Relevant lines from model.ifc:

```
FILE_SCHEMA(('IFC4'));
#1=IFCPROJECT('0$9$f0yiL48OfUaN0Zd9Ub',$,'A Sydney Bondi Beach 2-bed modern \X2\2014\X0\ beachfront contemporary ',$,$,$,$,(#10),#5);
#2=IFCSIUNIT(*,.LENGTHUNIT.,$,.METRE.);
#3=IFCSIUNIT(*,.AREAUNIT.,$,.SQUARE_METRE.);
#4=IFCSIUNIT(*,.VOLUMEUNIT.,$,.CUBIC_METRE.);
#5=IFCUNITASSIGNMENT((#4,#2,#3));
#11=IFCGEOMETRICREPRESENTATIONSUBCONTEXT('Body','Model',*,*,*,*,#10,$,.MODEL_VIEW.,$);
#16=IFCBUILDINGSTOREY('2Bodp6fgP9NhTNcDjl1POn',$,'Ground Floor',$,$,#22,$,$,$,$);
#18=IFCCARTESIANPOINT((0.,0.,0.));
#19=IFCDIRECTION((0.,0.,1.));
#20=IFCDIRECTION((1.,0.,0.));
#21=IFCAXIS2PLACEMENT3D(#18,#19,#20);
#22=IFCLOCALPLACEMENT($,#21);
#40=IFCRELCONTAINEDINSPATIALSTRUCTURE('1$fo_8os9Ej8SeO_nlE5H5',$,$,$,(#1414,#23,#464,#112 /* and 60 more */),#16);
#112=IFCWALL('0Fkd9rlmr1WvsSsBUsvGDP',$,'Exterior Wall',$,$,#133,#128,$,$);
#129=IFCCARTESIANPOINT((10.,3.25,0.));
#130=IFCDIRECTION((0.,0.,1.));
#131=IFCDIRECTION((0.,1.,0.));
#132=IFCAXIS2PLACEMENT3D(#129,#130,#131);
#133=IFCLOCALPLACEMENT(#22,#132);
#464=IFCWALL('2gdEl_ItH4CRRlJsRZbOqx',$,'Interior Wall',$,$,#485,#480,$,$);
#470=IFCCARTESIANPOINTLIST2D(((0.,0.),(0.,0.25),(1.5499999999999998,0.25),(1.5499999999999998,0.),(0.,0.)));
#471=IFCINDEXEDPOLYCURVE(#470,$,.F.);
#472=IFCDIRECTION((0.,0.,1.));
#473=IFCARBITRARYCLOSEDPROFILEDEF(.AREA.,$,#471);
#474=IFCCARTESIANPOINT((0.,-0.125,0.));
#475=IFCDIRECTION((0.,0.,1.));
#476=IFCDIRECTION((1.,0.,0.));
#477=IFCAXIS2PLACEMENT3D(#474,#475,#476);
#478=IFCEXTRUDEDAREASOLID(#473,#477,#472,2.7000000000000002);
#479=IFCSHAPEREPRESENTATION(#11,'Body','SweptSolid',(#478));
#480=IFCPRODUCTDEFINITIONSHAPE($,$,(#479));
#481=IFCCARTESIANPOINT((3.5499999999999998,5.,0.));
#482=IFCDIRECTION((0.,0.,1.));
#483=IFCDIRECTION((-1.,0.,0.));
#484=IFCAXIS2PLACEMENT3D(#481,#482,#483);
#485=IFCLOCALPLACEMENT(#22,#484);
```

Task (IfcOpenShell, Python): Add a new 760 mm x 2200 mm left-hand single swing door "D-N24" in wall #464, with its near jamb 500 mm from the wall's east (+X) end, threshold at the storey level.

```python
import numpy as np
import ifcopenshell
import ifcopenshell.api.feature
import ifcopenshell.api.geometry
import ifcopenshell.api.root
import ifcopenshell.api.spatial
import ifcopenshell.geom
import ifcopenshell.util.element
import ifcopenshell.util.placement
import ifcopenshell.util.representation
import ifcopenshell.util.shape
import ifcopenshell.util.unit

model = ifcopenshell.open("model.ifc")
unit_scale = ifcopenshell.util.unit.calculate_unit_scale(model)
settings = ifcopenshell.geom.settings()


def volume(element):
    """Net volume in cubic metres, openings subtracted."""
    shape = ifcopenshell.geom.create_shape(settings, element)
    return ifcopenshell.util.shape.get_volume(shape.geometry)


wall = model.by_guid("2gdEl_ItH4CRRlJsRZbOqx")
storey = ifcopenshell.util.element.get_container(wall, ifc_class="IfcBuildingStorey")
context = ifcopenshell.util.representation.get_context(model, "Model", "Body", "MODEL_VIEW")
before = volume(wall)

width, height, from_end, sill = 0.76, 2.2, 0.5, 0.0  # metres

# The wall runs along its own X axis, and the end named is its -X end.
wall_shape = ifcopenshell.geom.create_shape(settings, wall)
x, y, z = ifcopenshell.util.shape.get_vertices(wall_shape.geometry).T
start = x.min() + from_end
face, thickness = float(y.min()), float(y.max() - y.min())
wall_matrix = ifcopenshell.util.placement.get_local_placement(wall.ObjectPlacement)
level = ifcopenshell.util.placement.get_local_placement(storey.ObjectPlacement)[2, 3]


def in_wall(x, y):
    """Placement at x, y metres in the wall's axes, at sill height."""
    matrix = wall_matrix.copy()
    matrix[:, 3] = wall_matrix @ np.array([x / unit_scale, y / unit_scale, 0.0, 1.0])
    matrix[2, 3] = level + sill / unit_scale
    return matrix


# Opening: a box that overshoots both wall faces by 50 mm.
opening = ifcopenshell.api.root.create_entity(model, ifc_class="IfcOpeningElement", predefined_type="OPENING")
box = ifcopenshell.api.geometry.add_wall_representation(
    model, context=context, length=width, height=height, thickness=thickness + 0.1
)
ifcopenshell.api.geometry.assign_representation(model, product=opening, representation=box)
ifcopenshell.api.geometry.edit_object_placement(model, product=opening, matrix=in_wall(start, face - 0.05), is_si=False)
ifcopenshell.api.feature.add_feature(model, feature=opening, element=wall)

door = ifcopenshell.api.root.create_entity(model, ifc_class="IfcDoor", name="D-N24", predefined_type="DOOR")
door.OverallWidth, door.OverallHeight = width / unit_scale, height / unit_scale
door.OperationType = "SINGLE_SWING_LEFT"
body = ifcopenshell.api.geometry.add_door_representation(
    model,
    context=context,
    overall_width=door.OverallWidth,
    overall_height=door.OverallHeight,
    operation_type="SINGLE_SWING_LEFT",
    lining_properties={"LiningDepth": thickness / unit_scale, "ThresholdDepth": thickness / unit_scale},
)
ifcopenshell.api.geometry.assign_representation(model, product=door, representation=body)
ifcopenshell.api.spatial.assign_container(model, products=[door], relating_structure=storey)
ifcopenshell.api.feature.add_filling(model, opening=opening, element=door)

# The lining spans the wall, so the door starts at the wall face.
ifcopenshell.api.geometry.edit_object_placement(model, product=door, matrix=in_wall(start, face), is_si=False)

after = volume(wall)

print(f"wall volume {before:.3f} -> {after:.3f} m3")

model.write("model-out.ifc")
```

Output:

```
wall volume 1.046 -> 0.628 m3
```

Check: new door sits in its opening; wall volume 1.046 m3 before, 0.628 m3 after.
